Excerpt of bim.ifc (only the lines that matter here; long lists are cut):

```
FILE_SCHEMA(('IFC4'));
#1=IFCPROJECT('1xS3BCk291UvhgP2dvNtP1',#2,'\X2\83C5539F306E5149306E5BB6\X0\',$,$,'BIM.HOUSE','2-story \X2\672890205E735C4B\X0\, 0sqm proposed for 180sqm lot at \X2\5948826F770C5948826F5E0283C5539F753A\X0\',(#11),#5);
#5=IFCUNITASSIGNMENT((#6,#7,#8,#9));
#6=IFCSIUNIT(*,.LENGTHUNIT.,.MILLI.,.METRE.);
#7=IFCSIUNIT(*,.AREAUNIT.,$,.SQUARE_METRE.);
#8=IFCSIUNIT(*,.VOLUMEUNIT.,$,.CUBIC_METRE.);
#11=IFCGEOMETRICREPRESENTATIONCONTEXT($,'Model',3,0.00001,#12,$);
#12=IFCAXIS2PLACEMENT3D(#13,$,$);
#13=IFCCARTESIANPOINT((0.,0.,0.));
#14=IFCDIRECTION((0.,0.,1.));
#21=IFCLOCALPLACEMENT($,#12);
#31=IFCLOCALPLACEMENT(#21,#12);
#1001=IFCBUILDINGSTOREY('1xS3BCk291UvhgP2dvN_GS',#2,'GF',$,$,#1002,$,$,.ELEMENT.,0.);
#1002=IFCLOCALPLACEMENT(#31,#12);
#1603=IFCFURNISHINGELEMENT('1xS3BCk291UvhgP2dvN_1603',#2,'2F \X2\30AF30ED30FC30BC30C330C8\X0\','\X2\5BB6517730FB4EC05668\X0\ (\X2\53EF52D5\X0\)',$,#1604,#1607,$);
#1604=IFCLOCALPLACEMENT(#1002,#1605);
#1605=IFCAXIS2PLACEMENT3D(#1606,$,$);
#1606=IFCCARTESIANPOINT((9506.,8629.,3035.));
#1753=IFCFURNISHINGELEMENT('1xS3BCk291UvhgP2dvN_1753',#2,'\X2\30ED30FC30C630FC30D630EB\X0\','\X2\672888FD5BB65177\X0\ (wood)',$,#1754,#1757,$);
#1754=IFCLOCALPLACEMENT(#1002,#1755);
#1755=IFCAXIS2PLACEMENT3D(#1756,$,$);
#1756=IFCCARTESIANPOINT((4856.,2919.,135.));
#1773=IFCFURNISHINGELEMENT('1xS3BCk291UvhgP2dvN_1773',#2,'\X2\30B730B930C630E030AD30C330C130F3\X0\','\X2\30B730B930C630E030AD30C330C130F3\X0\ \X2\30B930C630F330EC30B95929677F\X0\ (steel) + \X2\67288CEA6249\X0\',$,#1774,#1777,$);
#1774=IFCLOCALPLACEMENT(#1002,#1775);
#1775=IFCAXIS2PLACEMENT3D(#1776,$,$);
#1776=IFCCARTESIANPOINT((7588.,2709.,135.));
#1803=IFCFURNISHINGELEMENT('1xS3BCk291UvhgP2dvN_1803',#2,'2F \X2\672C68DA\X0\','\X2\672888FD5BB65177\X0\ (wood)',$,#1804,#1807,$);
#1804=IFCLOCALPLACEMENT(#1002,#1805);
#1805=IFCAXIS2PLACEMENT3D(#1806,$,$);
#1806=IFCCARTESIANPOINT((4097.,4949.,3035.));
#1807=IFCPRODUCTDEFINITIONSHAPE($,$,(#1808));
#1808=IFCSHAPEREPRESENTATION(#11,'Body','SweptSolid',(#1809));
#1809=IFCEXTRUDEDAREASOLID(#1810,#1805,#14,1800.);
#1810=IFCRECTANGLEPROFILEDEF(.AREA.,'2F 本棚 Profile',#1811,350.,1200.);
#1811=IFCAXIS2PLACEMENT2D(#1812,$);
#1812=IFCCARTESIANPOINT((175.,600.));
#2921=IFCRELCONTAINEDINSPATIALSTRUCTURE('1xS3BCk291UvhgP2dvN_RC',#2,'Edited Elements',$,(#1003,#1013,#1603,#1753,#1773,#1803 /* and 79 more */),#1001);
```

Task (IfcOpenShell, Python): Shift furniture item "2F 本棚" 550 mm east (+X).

```python
import ifcopenshell
import ifcopenshell.api.geometry
import ifcopenshell.util.placement
import ifcopenshell.util.unit

model = ifcopenshell.open("bim.ifc")
unit_scale = ifcopenshell.util.unit.calculate_unit_scale(model)

item = model.by_guid("1xS3BCk291UvhgP2dvN_1803")
matrix = ifcopenshell.util.placement.get_local_placement(item.ObjectPlacement)
matrix[0, 3] += 0.55 / unit_scale
ifcopenshell.api.geometry.edit_object_placement(model, product=item, matrix=matrix, is_si=False)

print(ifcopenshell.util.placement.get_local_placement(item.ObjectPlacement).round(3) + 0.0)

model.write("bim_edited.ifc")
```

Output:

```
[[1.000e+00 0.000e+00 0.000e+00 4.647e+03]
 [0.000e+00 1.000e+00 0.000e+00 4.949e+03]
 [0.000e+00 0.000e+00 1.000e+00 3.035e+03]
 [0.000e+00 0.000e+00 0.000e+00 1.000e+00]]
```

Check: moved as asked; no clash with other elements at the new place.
